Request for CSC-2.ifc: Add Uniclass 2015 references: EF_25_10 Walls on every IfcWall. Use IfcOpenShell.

First a look at what the model holds.

```python
import ifcopenshell

model = ifcopenshell.open("CSC-2.ifc")
print(model.schema)
print("classifications:", [c.Name for c in model.by_type("IfcClassification")])
for ifc_class in ("IfcDoor", "IfcRoof", "IfcStair", "IfcWall", "IfcWindow"):
    print(ifc_class, len(model.by_type(ifc_class)))
```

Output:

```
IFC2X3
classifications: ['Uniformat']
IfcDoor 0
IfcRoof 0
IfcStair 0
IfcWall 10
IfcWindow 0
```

```python
import ifcopenshell
import ifcopenshell.api.classification

model = ifcopenshell.open("CSC-2.ifc")

# IFC2X3 requires Source and Edition and has no link from the project to the system.
system = model.create_entity("IfcClassification", Source="NBS", Edition="2015", Name="Uniclass 2015")

codes = {
    "IfcWall": ("EF_25_10", "Walls"),
}
for ifc_class, (code, name) in codes.items():
    products = model.by_type(ifc_class)
    ifcopenshell.api.classification.add_reference(
        model, products=products, classification=system, identification=code, name=name
    )
    print(code, len(products))

model.write("CSC-2_v2.ifc")
```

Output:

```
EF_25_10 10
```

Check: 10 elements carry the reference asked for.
